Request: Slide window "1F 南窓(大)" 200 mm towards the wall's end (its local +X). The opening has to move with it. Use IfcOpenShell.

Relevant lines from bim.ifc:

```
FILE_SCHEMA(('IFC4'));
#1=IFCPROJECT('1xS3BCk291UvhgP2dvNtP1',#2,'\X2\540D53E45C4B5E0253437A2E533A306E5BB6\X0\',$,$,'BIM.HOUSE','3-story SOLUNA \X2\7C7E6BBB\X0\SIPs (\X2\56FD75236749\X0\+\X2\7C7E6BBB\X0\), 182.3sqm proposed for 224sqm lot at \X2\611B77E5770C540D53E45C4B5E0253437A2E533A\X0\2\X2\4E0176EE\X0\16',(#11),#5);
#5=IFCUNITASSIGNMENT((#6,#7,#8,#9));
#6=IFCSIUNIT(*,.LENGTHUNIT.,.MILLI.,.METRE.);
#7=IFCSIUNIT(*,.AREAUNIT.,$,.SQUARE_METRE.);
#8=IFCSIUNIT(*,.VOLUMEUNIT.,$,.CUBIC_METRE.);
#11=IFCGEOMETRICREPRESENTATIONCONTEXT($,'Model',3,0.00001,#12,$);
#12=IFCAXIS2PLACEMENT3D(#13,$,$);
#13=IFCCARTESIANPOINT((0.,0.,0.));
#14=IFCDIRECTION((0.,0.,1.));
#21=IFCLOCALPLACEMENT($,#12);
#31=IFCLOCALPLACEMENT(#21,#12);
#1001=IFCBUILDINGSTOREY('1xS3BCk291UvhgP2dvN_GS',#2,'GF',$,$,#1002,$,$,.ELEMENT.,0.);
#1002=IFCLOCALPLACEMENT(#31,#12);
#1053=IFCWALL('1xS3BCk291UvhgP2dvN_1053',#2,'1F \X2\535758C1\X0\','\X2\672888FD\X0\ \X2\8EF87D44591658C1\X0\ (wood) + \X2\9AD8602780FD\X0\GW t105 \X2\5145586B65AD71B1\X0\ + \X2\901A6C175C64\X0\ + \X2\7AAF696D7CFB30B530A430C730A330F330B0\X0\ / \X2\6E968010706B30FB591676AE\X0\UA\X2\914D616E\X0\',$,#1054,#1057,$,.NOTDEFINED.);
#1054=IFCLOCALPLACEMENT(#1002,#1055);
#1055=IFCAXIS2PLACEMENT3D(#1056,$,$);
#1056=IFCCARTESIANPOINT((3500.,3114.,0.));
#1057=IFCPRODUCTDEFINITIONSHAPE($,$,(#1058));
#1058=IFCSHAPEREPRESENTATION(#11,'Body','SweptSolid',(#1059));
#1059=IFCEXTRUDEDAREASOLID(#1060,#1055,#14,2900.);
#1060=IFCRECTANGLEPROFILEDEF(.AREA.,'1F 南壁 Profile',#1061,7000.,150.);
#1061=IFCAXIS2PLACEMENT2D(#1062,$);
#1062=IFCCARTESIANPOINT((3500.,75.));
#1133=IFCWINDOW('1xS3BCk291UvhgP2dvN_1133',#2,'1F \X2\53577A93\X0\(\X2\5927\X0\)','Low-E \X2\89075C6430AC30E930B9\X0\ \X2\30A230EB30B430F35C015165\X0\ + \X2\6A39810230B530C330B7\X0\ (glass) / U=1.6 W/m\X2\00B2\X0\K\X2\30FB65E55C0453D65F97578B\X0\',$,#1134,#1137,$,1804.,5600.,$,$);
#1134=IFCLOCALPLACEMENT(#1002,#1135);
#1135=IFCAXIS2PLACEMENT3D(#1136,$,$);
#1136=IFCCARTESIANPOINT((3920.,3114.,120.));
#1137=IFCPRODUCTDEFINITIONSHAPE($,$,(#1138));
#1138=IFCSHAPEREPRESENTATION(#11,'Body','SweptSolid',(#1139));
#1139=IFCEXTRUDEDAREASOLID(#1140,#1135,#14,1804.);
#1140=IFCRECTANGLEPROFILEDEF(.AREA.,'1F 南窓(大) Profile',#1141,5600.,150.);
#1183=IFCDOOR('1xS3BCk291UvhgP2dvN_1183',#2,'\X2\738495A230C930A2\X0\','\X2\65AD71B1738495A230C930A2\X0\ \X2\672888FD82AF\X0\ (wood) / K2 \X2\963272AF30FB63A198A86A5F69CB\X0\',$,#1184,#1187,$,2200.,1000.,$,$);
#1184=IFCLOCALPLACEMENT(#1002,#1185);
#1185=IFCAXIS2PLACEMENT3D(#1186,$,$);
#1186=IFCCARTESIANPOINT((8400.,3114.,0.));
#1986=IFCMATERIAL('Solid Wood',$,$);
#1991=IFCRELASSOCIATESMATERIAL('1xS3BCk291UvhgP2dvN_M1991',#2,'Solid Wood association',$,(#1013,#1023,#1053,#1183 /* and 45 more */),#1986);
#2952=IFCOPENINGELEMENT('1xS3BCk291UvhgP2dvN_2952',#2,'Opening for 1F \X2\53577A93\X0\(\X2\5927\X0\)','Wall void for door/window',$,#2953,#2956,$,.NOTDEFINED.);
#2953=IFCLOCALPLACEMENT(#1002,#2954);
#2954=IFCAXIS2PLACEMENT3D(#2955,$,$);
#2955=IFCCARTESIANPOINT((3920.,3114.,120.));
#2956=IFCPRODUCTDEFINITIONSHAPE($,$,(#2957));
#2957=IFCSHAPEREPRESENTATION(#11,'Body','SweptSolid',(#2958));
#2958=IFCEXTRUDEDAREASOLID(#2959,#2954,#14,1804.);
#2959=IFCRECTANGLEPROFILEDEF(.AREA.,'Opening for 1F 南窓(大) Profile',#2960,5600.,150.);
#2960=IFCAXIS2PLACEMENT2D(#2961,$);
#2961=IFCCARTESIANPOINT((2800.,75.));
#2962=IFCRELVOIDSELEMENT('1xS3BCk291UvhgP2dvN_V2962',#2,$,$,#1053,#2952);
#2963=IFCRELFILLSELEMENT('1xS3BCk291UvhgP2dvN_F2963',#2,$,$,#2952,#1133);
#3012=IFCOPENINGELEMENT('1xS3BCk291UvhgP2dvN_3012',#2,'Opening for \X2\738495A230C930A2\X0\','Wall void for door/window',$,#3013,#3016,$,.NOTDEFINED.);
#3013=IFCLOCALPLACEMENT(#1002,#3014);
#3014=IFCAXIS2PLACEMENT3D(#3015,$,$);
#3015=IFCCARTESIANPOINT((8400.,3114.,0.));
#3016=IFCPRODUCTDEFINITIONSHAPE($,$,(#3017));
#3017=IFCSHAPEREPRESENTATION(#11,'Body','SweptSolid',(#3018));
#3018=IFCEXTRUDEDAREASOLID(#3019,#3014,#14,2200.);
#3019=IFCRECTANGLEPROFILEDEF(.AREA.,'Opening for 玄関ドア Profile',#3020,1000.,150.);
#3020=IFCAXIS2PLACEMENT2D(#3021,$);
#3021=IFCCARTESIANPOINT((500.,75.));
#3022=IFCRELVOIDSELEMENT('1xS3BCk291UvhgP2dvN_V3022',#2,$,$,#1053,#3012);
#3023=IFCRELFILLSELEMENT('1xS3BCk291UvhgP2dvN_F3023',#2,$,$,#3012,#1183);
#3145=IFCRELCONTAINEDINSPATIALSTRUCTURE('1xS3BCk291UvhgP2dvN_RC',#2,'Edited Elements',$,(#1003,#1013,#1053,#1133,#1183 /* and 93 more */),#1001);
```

```python
import ifcopenshell
import ifcopenshell.api.geometry
import ifcopenshell.util.placement
import ifcopenshell.util.unit

model = ifcopenshell.open("bim.ifc")
unit_scale = ifcopenshell.util.unit.calculate_unit_scale(model)

window = model.by_guid("1xS3BCk291UvhgP2dvN_1133")
opening = window.FillsVoids[0].RelatingOpeningElement
wall = opening.VoidsElements[0].RelatingBuildingElement

wall_matrix = ifcopenshell.util.placement.get_local_placement(wall.ObjectPlacement)
shift = wall_matrix[:3, 0] * 0.2 / unit_scale
before = ifcopenshell.util.placement.get_local_placement(window.ObjectPlacement)[:3, 3].copy()

# The window is not placed relative to its opening, so move both.
for product in (opening, window):
    matrix = ifcopenshell.util.placement.get_local_placement(product.ObjectPlacement)
    matrix[:3, 3] += shift
    ifcopenshell.api.geometry.edit_object_placement(model, product=product, matrix=matrix, is_si=False)

after = ifcopenshell.util.placement.get_local_placement(window.ObjectPlacement)[:3, 3]
print("window moved by", (after - before).round(3) + 0.0)

model.write("bim_v2.ifc")
```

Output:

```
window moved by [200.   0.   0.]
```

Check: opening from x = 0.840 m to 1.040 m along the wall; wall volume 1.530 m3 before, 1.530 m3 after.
